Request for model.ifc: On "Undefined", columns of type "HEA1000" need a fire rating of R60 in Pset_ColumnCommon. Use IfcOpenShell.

First a look at what the model holds.

```python
import ifcopenshell
import ifcopenshell.util.element

model = ifcopenshell.open("model.ifc")
print(model.schema)
storey = next(s for s in model.by_type("IfcBuildingStorey") if s.Name == "Undefined")
columns = [e for e in ifcopenshell.util.element.get_decomposition(storey) if e.is_a("IfcColumn")]
seen = {}
for e in columns:
    element_type = ifcopenshell.util.element.get_type(e)
    key = (element_type.Name if element_type != e and element_type else None, ifcopenshell.util.element.get_pset(e, "Pset_ColumnCommon", "FireRating"))
    seen[key] = seen.get(key, 0) + 1
for (name, value), count in sorted(seen.items(), key=str):
    print(count, "x", name, "|", value)
```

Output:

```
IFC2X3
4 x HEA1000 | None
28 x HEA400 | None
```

```python
import ifcopenshell
import ifcopenshell.api.pset
import ifcopenshell.util.element

model = ifcopenshell.open("model.ifc")

storey = next(s for s in model.by_type("IfcBuildingStorey") if s.Name == "Undefined")
columns = [e for e in ifcopenshell.util.element.get_decomposition(storey) if e.is_a("IfcColumn")]

count = 0
for e in columns:
    element_type = ifcopenshell.util.element.get_type(e)
    if element_type in (None, e) or element_type.Name != "HEA1000":
        continue
    found = ifcopenshell.util.element.get_pset(e, "Pset_ColumnCommon", should_inherit=False)
    if found:
        pset = model.by_id(found["id"])
        if len(ifcopenshell.util.element.get_elements_by_pset(pset)) > 1:
            pset = ifcopenshell.api.pset.unshare_pset(model, products=[e], pset=pset)[0]
    else:
        pset = ifcopenshell.api.pset.add_pset(model, product=e, name="Pset_ColumnCommon")
    ifcopenshell.api.pset.edit_pset(model, pset=pset, properties={"FireRating": "R60"})
    count += 1

print(count, "columns updated")

model.write("model_v2.ifc")
```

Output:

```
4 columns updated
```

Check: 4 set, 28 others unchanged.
